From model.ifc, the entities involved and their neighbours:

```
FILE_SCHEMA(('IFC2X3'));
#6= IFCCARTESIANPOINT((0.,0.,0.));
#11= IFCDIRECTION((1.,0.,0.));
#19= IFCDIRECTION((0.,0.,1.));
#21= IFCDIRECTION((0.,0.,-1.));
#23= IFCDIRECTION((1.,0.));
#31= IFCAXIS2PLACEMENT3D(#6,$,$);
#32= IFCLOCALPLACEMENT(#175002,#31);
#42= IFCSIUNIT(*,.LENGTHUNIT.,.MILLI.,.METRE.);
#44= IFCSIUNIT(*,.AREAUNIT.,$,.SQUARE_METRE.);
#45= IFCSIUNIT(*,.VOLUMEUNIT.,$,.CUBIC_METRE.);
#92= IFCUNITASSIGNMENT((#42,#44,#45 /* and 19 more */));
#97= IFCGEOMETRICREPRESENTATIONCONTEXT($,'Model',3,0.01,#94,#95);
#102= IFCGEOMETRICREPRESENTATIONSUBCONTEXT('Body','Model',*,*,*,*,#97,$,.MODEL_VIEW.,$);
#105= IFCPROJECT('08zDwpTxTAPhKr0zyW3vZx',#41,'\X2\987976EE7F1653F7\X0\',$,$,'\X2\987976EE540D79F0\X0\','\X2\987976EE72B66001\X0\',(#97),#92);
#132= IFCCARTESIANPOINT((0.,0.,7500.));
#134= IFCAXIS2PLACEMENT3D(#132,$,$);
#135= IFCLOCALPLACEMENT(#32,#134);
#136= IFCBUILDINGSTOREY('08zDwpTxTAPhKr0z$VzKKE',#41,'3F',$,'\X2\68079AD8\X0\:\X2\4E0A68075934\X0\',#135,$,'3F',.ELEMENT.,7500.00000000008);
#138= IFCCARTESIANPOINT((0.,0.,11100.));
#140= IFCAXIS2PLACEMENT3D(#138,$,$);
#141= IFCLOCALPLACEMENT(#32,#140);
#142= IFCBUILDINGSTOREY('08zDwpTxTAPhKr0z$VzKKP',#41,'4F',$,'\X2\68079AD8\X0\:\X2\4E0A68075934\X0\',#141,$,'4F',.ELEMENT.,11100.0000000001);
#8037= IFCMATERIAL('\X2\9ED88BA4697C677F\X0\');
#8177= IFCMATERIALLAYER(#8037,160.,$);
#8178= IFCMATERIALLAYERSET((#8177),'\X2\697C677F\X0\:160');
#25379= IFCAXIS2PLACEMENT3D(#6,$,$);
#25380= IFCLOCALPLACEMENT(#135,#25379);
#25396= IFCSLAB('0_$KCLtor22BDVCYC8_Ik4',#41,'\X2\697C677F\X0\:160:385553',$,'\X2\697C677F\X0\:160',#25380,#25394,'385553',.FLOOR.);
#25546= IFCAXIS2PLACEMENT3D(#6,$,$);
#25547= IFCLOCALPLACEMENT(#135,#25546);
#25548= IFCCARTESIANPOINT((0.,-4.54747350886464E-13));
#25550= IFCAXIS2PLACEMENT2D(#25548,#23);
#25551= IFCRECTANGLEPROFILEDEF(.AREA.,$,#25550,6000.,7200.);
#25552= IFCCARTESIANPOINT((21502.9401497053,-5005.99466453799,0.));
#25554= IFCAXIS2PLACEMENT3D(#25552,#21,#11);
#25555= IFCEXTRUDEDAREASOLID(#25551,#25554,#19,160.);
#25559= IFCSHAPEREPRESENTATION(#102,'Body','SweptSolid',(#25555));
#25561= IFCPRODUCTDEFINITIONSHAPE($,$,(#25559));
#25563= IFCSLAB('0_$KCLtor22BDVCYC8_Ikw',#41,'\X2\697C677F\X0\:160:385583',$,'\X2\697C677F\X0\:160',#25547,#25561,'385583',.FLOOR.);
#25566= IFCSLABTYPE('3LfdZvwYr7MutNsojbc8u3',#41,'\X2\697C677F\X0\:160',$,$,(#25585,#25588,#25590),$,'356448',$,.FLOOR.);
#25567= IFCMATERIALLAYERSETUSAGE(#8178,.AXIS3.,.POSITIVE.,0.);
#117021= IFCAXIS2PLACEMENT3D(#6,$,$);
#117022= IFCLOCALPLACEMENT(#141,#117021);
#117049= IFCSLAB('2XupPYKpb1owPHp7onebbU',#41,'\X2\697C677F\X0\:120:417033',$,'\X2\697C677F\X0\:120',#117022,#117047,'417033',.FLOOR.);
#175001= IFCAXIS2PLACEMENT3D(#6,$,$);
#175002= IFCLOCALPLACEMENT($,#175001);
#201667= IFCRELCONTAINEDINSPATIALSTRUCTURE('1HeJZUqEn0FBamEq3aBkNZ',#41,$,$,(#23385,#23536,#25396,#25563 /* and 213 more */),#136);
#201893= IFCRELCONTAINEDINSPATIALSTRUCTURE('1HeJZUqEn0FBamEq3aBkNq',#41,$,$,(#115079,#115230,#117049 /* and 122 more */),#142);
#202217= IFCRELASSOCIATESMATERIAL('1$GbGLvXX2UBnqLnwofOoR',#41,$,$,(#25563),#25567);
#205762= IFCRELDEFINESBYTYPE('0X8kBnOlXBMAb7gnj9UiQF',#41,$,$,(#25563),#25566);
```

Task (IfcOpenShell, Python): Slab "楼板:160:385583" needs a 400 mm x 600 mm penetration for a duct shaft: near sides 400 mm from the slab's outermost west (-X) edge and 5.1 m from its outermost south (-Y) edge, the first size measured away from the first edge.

```python
import numpy as np
import ifcopenshell
import ifcopenshell.api.feature
import ifcopenshell.api.geometry
import ifcopenshell.api.root
import ifcopenshell.geom
import ifcopenshell.util.placement
import ifcopenshell.util.representation
import ifcopenshell.util.shape
import ifcopenshell.util.unit

model = ifcopenshell.open("model.ifc")
unit_scale = ifcopenshell.util.unit.calculate_unit_scale(model)
settings = ifcopenshell.geom.settings()


def volume(element):
    """Net volume in cubic metres, openings subtracted."""
    shape = ifcopenshell.geom.create_shape(settings, element)
    return ifcopenshell.util.shape.get_volume(shape.geometry)


slab = model.by_guid("0_$KCLtor22BDVCYC8_Ikw")
before = volume(slab)

# Extent in the slab's own axes, in metres. The edges named are its -X and -Y sides.
slab_shape = ifcopenshell.geom.create_shape(settings, slab)
vertices = ifcopenshell.util.shape.get_vertices(slab_shape.geometry)
x_min, y_min, bottom = vertices.min(axis=0)
top = vertices[:, 2].max()

opening = ifcopenshell.api.root.create_entity(model, ifc_class="IfcOpeningElement", name="Duct shaft opening")
context = ifcopenshell.util.representation.get_context(model, "Model", "Body", "MODEL_VIEW")
width, depth = 0.4, 0.6
outline = [(0.0, 0.0), (width, 0.0), (width, depth), (0.0, depth), (0.0, 0.0)]
# Overshoot both faces by 50 mm so the cut is clean.
shape = ifcopenshell.api.geometry.add_slab_representation(
    model, context=context, depth=top - bottom + 0.1, polyline=outline
)
ifcopenshell.api.geometry.assign_representation(model, product=opening, representation=shape)

matrix = ifcopenshell.util.placement.get_local_placement(slab.ObjectPlacement)
matrix[:, 3] = matrix @ np.append(np.array([x_min + 0.4, y_min + 5.1, bottom - 0.05]) / unit_scale, 1.0)
ifcopenshell.api.geometry.edit_object_placement(model, product=opening, matrix=matrix, is_si=False)
ifcopenshell.api.feature.add_feature(model, feature=opening, element=slab)

after = volume(slab)

print(f"slab volume {before:.3f} -> {after:.3f} m3")

model.write("model_updated.ifc")
```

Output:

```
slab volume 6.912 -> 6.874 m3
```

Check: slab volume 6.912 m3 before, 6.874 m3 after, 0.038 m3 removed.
